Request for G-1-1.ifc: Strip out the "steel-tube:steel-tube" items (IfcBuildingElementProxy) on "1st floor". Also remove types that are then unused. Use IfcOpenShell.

First a look at what the model holds.

```python
import ifcopenshell
import ifcopenshell.util.element

model = ifcopenshell.open("G-1-1.ifc")
print(model.schema)
storey = next(s for s in model.by_type("IfcBuildingStorey") if s.Name == "1st floor")
proxies = [e for e in ifcopenshell.util.element.get_decomposition(storey) if e.is_a("IfcBuildingElementProxy")]
seen = {}
for e in proxies:
    element_type = ifcopenshell.util.element.get_type(e)
    name = element_type.Name if element_type not in (None, e) else None
    seen[name] = seen.get(name, 0) + 1
for name, count in sorted(seen.items(), key=str):
    print(count, "x", name)
```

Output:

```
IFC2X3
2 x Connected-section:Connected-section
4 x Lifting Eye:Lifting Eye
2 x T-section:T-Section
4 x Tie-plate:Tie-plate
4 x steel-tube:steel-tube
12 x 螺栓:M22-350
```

```python
import ifcopenshell
import ifcopenshell.api.root
import ifcopenshell.util.element

model = ifcopenshell.open("G-1-1.ifc")

storey = next(s for s in model.by_type("IfcBuildingStorey") if s.Name == "1st floor")
proxies = [e for e in ifcopenshell.util.element.get_decomposition(storey) if e.is_a("IfcBuildingElementProxy")]
targets = [e for e in proxies if (t := ifcopenshell.util.element.get_type(e)) not in (None, e) and t.Name == "steel-tube:steel-tube"]
types = {ifcopenshell.util.element.get_type(e) for e in targets} - {None, *targets}

for e in targets:
    ifcopenshell.api.root.remove_product(model, product=e)
print(len(targets), "removed")

unused = [t for t in types if not ifcopenshell.util.element.get_types(t)]
for t in unused:
    ifcopenshell.api.root.remove_product(model, product=t)
print(len(unused), "unused types removed")

model.write("G-1-1-out.ifc")
```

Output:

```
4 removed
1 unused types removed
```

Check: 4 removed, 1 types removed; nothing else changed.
